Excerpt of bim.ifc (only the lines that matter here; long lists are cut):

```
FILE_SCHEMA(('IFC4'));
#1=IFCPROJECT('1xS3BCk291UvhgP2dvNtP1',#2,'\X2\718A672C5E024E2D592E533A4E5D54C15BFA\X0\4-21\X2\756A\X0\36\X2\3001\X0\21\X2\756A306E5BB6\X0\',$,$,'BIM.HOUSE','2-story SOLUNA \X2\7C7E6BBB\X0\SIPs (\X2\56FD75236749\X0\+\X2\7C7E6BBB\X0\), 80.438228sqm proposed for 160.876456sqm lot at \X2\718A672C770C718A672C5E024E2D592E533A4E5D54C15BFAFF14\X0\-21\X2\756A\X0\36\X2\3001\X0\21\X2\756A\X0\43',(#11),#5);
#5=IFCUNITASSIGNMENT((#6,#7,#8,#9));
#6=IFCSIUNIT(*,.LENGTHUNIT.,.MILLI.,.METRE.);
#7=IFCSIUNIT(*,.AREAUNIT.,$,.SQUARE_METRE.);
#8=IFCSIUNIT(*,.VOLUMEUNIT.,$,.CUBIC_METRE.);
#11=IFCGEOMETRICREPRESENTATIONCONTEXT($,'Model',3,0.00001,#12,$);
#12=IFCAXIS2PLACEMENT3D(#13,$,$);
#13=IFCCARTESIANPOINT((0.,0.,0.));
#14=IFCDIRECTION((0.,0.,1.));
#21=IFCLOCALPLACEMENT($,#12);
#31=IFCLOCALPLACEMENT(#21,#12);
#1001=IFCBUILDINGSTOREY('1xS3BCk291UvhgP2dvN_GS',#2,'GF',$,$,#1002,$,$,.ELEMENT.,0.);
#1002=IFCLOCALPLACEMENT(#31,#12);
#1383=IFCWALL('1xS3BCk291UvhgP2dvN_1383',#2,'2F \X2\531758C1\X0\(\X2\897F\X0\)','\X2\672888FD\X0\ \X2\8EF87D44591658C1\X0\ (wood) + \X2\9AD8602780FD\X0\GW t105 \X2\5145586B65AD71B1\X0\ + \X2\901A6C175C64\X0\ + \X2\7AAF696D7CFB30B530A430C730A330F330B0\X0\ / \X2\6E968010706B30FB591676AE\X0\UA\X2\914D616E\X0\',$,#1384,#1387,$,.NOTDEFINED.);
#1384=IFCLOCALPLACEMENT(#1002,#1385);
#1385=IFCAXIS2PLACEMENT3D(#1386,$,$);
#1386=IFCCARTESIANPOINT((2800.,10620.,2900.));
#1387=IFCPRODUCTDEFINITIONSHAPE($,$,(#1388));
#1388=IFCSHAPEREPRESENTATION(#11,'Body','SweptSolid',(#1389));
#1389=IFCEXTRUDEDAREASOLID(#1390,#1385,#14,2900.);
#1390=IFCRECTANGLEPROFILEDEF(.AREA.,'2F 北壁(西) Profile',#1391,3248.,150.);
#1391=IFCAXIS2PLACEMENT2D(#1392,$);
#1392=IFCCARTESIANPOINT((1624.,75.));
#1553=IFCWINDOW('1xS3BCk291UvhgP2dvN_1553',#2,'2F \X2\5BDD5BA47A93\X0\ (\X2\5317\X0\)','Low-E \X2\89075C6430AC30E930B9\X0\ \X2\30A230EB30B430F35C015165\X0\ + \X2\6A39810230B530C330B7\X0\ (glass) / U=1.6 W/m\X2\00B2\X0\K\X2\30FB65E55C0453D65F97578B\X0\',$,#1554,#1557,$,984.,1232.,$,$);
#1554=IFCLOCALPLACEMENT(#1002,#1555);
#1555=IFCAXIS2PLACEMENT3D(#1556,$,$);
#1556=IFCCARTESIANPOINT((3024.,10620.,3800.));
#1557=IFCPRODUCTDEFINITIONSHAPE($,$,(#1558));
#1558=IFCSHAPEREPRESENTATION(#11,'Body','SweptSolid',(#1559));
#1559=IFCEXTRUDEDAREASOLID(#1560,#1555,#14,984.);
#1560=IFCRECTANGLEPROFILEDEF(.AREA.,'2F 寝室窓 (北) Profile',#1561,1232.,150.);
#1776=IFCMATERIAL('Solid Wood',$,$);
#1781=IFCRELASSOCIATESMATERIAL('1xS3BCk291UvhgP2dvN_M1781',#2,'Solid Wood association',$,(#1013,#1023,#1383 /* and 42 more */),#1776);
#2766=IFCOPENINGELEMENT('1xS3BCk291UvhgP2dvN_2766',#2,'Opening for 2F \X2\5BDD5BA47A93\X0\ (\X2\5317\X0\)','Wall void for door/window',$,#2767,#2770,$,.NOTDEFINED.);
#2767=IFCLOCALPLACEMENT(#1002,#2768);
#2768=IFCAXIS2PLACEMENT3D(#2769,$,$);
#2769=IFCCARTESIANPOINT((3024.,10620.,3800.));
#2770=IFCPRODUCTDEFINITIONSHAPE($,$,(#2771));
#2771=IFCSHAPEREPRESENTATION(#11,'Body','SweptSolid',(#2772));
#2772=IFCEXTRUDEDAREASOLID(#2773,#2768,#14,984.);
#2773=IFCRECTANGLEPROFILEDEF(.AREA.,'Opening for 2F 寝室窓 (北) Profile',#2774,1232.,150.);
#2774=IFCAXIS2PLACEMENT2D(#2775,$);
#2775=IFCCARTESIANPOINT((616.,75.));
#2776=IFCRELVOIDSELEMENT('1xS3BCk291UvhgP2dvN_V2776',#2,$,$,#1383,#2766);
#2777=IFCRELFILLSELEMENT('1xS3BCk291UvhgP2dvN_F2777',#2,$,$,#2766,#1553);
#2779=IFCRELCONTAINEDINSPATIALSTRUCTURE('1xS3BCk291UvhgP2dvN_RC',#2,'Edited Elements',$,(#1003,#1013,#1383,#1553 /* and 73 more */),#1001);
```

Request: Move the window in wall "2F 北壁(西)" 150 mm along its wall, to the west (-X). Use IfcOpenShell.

```python
import ifcopenshell
import ifcopenshell.api.geometry
import ifcopenshell.util.placement

model = ifcopenshell.open("bim.ifc")

window = model.by_id(1553)
opening = window.FillsVoids[0].RelatingOpeningElement
wall = opening.VoidsElements[0].RelatingBuildingElement

wall_matrix = ifcopenshell.util.placement.get_local_placement(wall.ObjectPlacement)
shift = wall_matrix[:3, 0] * -150.0
before = ifcopenshell.util.placement.get_local_placement(window.ObjectPlacement)[:3, 3].copy()

# The window is not placed relative to its opening, so move both.
for product in (opening, window):
    matrix = ifcopenshell.util.placement.get_local_placement(product.ObjectPlacement)
    matrix[:3, 3] += shift
    ifcopenshell.api.geometry.edit_object_placement(model, product=product, matrix=matrix, is_si=False)

after = ifcopenshell.util.placement.get_local_placement(window.ObjectPlacement)[:3, 3]
print("window moved by", (after - before).round(3) + 0.0)

model.write("bim_v2.ifc")
```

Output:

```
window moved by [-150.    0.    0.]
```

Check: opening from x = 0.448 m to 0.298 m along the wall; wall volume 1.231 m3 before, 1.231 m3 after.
